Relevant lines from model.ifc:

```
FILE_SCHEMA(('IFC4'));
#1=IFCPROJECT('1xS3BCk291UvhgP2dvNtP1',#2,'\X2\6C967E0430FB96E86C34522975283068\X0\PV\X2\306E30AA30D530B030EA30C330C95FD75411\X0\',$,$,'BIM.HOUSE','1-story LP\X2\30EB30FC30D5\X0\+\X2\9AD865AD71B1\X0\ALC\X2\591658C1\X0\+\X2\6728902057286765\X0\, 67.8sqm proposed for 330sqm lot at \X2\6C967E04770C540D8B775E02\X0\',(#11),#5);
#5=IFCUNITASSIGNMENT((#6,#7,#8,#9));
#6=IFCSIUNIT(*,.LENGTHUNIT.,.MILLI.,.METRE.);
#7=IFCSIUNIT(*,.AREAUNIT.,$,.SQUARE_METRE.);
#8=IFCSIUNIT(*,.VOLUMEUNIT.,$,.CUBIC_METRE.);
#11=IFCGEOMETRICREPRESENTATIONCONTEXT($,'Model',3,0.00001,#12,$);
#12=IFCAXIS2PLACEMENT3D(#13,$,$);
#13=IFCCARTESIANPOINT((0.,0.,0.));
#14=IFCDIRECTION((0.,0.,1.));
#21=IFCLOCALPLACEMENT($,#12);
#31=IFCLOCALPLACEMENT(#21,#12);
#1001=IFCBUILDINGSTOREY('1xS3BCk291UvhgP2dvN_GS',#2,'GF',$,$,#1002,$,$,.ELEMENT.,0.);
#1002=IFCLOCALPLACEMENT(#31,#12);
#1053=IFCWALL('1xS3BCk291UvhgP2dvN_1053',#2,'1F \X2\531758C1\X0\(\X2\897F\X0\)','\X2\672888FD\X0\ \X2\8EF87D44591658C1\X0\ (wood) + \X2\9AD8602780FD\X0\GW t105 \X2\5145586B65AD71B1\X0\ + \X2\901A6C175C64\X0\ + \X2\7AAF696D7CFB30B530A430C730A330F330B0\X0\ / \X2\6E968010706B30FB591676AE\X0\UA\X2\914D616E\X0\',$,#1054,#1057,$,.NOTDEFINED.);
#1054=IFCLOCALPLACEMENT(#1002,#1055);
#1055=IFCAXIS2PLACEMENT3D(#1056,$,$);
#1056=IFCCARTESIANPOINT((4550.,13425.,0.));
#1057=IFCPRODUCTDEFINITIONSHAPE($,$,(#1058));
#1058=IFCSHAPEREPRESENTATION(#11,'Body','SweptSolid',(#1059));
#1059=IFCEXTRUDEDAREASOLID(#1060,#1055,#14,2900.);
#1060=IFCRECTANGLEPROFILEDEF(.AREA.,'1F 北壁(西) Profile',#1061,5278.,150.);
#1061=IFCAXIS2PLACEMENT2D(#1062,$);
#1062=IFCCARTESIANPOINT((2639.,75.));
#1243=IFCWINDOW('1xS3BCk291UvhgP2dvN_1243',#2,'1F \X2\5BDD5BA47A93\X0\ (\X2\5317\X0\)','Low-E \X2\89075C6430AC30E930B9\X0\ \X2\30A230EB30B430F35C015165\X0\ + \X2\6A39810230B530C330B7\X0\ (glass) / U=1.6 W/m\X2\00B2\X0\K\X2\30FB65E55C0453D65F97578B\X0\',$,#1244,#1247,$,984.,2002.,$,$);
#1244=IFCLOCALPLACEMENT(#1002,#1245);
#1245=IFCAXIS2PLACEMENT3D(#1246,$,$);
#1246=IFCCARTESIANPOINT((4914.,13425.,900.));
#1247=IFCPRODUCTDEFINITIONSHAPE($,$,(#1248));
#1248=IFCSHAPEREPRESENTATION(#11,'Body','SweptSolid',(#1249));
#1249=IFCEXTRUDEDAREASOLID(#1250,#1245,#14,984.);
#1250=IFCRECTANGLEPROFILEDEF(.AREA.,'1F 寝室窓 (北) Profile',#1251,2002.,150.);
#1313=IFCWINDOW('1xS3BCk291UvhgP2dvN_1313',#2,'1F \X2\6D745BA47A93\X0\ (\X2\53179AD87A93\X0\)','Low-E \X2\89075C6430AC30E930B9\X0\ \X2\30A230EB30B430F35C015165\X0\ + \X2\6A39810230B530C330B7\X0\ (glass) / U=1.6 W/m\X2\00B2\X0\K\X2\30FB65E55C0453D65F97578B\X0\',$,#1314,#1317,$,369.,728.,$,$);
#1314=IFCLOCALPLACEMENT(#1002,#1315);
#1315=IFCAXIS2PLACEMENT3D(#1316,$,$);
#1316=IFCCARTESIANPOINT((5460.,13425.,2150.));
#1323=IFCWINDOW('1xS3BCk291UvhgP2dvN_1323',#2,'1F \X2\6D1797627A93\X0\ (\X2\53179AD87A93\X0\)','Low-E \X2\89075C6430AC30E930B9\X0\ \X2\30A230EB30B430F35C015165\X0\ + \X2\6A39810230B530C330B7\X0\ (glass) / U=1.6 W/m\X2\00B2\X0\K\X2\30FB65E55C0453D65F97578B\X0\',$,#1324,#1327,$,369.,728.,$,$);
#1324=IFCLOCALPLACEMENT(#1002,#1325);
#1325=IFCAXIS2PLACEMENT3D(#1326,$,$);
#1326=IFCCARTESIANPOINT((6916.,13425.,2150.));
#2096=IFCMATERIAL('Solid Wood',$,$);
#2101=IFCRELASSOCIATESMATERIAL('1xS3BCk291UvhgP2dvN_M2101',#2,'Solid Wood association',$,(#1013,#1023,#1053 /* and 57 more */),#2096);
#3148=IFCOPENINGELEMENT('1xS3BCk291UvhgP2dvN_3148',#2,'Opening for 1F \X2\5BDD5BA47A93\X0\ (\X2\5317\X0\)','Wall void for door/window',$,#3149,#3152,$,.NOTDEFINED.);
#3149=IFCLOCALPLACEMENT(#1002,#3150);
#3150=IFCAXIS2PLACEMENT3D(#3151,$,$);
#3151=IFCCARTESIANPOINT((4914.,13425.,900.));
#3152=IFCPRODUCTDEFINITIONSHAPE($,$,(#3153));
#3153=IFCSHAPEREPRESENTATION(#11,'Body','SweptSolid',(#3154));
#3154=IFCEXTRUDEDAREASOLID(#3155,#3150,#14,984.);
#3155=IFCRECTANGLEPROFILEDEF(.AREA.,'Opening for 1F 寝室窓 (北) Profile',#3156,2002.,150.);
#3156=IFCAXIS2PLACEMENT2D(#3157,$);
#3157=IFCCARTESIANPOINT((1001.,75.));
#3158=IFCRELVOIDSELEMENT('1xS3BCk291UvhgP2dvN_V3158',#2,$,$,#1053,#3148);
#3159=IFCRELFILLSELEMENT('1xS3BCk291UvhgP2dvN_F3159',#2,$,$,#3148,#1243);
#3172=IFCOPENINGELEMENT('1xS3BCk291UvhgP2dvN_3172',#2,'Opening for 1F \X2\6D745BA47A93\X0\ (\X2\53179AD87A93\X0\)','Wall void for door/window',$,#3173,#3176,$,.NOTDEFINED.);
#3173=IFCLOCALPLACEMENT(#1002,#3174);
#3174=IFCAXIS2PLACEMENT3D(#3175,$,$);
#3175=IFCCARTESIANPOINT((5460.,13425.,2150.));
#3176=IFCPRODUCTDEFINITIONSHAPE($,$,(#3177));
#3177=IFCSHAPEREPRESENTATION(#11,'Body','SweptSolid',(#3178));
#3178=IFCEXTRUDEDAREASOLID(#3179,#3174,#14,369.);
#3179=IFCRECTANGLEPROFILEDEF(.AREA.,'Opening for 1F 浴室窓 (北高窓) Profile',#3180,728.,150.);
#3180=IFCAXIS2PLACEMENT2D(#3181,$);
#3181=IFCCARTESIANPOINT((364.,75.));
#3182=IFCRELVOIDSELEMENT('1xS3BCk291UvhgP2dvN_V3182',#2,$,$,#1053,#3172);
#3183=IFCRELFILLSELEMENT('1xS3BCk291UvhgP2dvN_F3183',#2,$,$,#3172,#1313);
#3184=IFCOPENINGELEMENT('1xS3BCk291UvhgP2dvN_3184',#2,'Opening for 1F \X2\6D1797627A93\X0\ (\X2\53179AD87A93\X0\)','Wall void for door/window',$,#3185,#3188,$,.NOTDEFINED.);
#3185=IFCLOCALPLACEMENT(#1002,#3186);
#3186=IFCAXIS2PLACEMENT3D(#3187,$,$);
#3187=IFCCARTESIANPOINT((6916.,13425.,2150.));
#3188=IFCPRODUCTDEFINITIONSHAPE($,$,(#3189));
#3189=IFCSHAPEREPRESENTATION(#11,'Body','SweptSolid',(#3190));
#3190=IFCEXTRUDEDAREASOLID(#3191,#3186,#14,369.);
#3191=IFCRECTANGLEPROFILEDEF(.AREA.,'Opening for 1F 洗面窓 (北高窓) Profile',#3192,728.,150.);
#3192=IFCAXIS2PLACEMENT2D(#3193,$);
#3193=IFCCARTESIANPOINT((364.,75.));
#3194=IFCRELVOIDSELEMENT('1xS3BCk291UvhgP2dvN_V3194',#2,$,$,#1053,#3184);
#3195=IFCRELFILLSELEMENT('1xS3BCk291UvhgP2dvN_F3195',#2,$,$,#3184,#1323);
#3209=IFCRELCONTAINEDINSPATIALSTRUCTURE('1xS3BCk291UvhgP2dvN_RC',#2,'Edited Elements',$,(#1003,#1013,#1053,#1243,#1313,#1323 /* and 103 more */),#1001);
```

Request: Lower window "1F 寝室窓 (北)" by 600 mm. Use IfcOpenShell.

```python
import numpy as np
import ifcopenshell
import ifcopenshell.api.geometry
import ifcopenshell.util.placement
import ifcopenshell.util.unit

model = ifcopenshell.open("model.ifc")
unit_scale = ifcopenshell.util.unit.calculate_unit_scale(model)

window = model.by_guid("1xS3BCk291UvhgP2dvN_1243")
opening = window.FillsVoids[0].RelatingOpeningElement
dz = -0.6 / unit_scale

shift = np.array([0.0, 0.0, dz])
# The window is not placed relative to its opening, so move both.
for product in (opening, window):
    matrix = ifcopenshell.util.placement.get_local_placement(product.ObjectPlacement)
    matrix[:3, 3] += shift
    ifcopenshell.api.geometry.edit_object_placement(model, product=product, matrix=matrix, is_si=False)

print(f"moved by {dz * unit_scale:+.3f} m")

model.write("model-out.ifc")
```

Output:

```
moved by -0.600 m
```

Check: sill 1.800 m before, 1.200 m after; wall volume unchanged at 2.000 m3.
